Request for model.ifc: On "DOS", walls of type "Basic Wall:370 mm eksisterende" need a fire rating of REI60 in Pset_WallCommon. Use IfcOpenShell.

First a look at what the model holds.

```python
import ifcopenshell
import ifcopenshell.util.element

model = ifcopenshell.open("model.ifc")
print(model.schema)
storey = next(s for s in model.by_type("IfcBuildingStorey") if s.Name == "DOS")
walls = [e for e in ifcopenshell.util.element.get_decomposition(storey) if e.is_a("IfcWall")]
seen = {}
for e in walls:
    element_type = ifcopenshell.util.element.get_type(e)
    key = (element_type.Name if element_type != e and element_type else None, ifcopenshell.util.element.get_pset(e, "Pset_WallCommon", "FireRating"))
    seen[key] = seen.get(key, 0) + 1
for (name, value), count in sorted(seen.items(), key=str):
    print(count, "x", name, "|", value)
```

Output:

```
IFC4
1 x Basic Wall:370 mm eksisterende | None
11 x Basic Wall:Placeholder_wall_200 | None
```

```python
import ifcopenshell
import ifcopenshell.api.pset
import ifcopenshell.util.element

model = ifcopenshell.open("model.ifc")

storey = next(s for s in model.by_type("IfcBuildingStorey") if s.Name == "DOS")
walls = [e for e in ifcopenshell.util.element.get_decomposition(storey) if e.is_a("IfcWall")]

count = 0
for e in walls:
    element_type = ifcopenshell.util.element.get_type(e)
    if element_type in (None, e) or element_type.Name != "Basic Wall:370 mm eksisterende":
        continue
    # add_pset returns the element's existing set when there is one.
    pset = ifcopenshell.api.pset.add_pset(model, product=e, name="Pset_WallCommon")
    ifcopenshell.api.pset.edit_pset(model, pset=pset, properties={"FireRating": "REI60"})
    count += 1

print(count, "walls updated")

model.write("model_v2.ifc")
```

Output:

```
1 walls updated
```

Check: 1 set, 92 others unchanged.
